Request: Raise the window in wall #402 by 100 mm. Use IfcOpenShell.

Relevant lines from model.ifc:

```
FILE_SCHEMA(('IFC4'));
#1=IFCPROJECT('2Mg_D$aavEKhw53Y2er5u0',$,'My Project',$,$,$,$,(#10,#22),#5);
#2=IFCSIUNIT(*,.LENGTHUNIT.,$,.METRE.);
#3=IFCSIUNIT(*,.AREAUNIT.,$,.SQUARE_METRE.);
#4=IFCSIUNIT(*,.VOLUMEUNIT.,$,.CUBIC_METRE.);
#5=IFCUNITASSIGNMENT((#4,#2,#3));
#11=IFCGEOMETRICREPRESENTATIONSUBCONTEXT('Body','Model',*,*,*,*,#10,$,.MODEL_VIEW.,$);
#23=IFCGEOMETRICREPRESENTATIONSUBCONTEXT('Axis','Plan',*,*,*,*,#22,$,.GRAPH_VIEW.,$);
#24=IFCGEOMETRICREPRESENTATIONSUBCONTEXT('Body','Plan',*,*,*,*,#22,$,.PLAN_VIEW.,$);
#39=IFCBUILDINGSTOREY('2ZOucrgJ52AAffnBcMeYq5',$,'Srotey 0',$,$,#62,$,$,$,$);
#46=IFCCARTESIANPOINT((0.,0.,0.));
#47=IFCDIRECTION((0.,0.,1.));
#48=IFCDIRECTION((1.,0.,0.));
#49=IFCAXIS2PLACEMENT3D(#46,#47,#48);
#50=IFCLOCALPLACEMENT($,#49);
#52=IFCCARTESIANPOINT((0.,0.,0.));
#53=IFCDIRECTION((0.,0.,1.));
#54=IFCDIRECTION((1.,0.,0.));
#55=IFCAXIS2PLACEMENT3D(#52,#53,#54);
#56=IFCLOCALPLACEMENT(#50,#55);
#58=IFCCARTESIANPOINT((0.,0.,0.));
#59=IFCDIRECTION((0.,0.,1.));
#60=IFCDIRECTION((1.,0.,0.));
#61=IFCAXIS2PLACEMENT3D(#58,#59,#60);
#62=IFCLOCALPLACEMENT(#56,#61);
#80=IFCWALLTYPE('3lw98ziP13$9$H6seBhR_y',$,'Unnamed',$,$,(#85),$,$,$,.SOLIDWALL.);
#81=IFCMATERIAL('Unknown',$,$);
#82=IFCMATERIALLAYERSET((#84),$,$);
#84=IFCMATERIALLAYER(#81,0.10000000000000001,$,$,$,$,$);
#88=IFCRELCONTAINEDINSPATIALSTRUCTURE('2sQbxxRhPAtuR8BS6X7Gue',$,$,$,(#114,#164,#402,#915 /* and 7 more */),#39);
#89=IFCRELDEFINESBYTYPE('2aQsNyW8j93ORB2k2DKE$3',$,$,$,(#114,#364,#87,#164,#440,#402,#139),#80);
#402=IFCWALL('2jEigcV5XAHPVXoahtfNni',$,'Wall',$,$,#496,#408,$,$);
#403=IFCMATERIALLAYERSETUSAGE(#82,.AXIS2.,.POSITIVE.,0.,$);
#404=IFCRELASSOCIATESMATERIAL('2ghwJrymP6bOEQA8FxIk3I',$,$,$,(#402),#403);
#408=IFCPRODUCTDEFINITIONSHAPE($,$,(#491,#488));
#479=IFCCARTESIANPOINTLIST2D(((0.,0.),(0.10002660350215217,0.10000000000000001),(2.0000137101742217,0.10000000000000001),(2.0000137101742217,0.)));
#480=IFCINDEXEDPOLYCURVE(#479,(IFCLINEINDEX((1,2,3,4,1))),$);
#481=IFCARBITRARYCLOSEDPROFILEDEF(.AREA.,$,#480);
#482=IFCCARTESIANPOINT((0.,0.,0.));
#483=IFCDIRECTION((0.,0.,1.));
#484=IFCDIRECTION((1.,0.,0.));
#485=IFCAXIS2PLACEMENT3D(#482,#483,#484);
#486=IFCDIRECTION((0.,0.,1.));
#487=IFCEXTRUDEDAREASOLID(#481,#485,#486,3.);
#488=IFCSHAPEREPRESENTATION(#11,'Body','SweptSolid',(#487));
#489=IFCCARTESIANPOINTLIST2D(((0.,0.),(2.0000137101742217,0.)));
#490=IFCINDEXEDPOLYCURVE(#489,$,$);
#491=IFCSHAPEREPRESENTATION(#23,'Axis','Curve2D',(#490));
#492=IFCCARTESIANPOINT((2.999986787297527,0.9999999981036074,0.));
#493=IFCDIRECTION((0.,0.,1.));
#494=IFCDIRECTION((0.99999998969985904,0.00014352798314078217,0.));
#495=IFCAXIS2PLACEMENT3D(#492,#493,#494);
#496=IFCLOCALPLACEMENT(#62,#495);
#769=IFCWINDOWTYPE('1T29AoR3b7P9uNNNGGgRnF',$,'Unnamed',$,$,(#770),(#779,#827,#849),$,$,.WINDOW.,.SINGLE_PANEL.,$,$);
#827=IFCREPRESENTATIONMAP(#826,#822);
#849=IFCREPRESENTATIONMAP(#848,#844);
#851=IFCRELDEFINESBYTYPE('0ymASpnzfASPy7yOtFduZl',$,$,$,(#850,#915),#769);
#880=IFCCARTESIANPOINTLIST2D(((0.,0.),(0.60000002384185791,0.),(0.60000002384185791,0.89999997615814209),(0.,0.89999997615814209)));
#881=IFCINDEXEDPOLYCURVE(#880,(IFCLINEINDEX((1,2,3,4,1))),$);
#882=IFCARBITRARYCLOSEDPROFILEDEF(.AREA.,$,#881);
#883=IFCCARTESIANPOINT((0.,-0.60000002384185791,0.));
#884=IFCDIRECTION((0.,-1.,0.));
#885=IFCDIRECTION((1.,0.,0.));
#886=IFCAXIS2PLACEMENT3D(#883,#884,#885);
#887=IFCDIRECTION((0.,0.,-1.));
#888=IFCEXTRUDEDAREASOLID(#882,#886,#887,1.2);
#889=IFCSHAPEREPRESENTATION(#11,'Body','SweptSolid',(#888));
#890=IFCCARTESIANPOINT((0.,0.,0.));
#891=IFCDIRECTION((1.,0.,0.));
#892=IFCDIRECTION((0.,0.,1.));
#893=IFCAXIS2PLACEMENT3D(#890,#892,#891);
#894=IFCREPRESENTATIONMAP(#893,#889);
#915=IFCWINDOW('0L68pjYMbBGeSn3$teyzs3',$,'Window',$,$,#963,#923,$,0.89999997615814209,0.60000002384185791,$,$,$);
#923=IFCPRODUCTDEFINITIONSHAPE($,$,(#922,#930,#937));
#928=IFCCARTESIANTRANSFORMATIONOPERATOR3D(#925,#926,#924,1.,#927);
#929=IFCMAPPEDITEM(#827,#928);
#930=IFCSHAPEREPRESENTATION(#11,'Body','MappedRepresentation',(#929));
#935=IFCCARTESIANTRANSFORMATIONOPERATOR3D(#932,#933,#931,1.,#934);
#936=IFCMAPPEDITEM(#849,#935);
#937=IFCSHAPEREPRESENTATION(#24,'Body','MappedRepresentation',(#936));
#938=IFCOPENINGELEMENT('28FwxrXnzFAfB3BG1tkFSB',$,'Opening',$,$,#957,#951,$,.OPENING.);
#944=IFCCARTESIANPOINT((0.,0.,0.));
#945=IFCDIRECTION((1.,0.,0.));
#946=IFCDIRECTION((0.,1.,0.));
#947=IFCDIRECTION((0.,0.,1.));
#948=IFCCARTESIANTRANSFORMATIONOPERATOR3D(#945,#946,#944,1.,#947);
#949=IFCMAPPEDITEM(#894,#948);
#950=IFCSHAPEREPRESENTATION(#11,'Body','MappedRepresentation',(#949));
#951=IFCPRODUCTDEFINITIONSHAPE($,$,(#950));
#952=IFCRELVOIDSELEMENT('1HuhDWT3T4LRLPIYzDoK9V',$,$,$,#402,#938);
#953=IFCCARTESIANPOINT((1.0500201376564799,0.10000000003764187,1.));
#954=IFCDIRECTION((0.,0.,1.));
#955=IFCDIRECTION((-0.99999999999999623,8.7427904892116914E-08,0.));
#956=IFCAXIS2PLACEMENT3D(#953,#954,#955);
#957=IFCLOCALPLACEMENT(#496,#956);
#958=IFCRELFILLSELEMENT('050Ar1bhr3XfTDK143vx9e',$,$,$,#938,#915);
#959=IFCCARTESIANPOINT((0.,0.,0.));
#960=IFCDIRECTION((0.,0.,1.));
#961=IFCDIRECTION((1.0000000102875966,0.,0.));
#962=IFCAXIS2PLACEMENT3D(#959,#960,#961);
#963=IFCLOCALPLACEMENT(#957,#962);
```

```python
import numpy as np
import ifcopenshell
import ifcopenshell.api.geometry
import ifcopenshell.util.placement
import ifcopenshell.util.unit

model = ifcopenshell.open("model.ifc")
unit_scale = ifcopenshell.util.unit.calculate_unit_scale(model)

window = model.by_guid("0L68pjYMbBGeSn3$teyzs3")
opening = window.FillsVoids[0].RelatingOpeningElement
dz = 0.1 / unit_scale

shift = np.array([0.0, 0.0, dz])
# The window is placed relative to its opening, so it follows when the opening moves.
matrix = ifcopenshell.util.placement.get_local_placement(opening.ObjectPlacement)
matrix[:3, 3] += shift
ifcopenshell.api.geometry.edit_object_placement(
    model, product=opening, matrix=matrix, is_si=False, should_transform_children=True
)

print(f"moved by {dz * unit_scale:+.3f} m")

model.write("model_rev.ifc")
```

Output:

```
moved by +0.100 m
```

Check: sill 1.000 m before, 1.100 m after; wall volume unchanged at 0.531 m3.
